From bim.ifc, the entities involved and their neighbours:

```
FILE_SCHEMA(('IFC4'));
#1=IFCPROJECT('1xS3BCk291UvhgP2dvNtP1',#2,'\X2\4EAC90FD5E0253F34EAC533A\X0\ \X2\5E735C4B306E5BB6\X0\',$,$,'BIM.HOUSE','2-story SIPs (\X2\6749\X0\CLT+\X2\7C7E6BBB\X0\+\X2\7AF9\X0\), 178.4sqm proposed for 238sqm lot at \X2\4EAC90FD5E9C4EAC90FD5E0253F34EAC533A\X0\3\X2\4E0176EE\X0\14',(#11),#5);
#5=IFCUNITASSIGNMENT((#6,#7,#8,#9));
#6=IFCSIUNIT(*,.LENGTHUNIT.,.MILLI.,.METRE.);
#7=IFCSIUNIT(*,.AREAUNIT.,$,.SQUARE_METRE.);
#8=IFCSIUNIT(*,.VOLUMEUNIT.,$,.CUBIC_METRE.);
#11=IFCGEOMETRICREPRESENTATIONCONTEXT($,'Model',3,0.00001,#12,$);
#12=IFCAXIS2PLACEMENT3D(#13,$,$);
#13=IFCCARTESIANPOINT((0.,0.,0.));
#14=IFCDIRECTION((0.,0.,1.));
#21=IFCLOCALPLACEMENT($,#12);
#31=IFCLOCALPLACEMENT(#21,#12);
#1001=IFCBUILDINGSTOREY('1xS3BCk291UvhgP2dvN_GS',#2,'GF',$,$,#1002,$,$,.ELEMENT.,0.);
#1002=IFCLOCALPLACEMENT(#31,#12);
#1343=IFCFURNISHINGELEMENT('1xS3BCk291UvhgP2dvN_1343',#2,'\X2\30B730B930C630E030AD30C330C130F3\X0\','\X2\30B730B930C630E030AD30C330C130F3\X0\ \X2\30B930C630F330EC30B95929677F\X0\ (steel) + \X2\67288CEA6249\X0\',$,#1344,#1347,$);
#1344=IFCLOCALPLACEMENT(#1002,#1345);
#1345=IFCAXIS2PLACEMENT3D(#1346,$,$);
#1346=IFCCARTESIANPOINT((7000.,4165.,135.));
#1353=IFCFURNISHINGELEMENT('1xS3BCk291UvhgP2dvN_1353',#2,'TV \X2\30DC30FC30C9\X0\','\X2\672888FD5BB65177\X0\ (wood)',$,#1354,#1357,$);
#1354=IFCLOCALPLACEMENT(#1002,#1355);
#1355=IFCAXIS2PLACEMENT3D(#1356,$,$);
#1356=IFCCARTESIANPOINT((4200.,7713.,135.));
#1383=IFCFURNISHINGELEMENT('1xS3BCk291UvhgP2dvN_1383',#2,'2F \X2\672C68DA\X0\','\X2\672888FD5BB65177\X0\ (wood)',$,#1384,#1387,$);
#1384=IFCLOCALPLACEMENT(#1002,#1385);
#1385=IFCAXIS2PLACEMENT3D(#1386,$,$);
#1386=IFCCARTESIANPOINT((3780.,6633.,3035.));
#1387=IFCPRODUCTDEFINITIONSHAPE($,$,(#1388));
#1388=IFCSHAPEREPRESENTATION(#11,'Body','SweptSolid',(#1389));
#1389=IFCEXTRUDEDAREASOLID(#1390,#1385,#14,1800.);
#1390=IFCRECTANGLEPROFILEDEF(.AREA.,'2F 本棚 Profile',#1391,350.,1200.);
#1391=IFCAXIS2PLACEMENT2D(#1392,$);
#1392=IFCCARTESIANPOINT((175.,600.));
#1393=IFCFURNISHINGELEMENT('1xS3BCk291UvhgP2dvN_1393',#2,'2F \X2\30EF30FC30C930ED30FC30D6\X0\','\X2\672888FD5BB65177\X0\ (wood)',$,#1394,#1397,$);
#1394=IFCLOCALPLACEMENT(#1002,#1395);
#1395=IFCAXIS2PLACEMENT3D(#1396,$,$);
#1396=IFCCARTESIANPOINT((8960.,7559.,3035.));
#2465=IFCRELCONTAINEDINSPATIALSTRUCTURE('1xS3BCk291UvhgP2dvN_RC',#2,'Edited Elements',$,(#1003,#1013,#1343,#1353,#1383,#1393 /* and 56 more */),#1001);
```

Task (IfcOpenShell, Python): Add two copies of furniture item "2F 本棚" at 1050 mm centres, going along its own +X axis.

```python
import ifcopenshell
import ifcopenshell.api.geometry
import ifcopenshell.api.root
import ifcopenshell.util.element
import ifcopenshell.util.placement
import ifcopenshell.util.unit

model = ifcopenshell.open("bim.ifc")
unit_scale = ifcopenshell.util.unit.calculate_unit_scale(model)


def reuse_history(source, copy):
    """copy_class also copies each property set's owner history, people and application; keep the originals."""
    for rel in copy.IsDefinedBy:
        if rel.is_a("IfcRelDefinesByProperties") and (history := rel.RelatingPropertyDefinition.OwnerHistory):
            rel.RelatingPropertyDefinition.OwnerHistory = source.OwnerHistory
            ifcopenshell.util.element.remove_deep2(model, history)


source = model.by_guid("1xS3BCk291UvhgP2dvN_1383")
base = ifcopenshell.util.placement.get_local_placement(source.ObjectPlacement)
step = base[:3, 0] * 1.05 / unit_scale

for i in range(1, 3):
    copy = ifcopenshell.api.root.copy_class(model, product=source)
    copy.Representation = ifcopenshell.util.element.copy_deep(
        model, source.Representation, exclude=["IfcGeometricRepresentationContext", "IfcRepresentationMap"]
    )
    reuse_history(source, copy)
    matrix = base.copy()
    matrix[:3, 3] += i * step
    print("added at", matrix[:3, 3].round(3) + 0.0)
    ifcopenshell.api.geometry.edit_object_placement(model, product=copy, matrix=matrix, is_si=False)

model.write("bim_rev.ifc")
```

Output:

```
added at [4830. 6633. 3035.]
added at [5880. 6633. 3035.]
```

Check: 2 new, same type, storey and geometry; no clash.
